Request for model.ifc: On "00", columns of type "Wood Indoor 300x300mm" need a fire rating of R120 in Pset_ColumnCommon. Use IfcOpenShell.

First a look at what the model holds.

```python
import ifcopenshell
import ifcopenshell.util.element

model = ifcopenshell.open("model.ifc")
print(model.schema)
storey = next(s for s in model.by_type("IfcBuildingStorey") if s.Name == "00")
columns = [e for e in ifcopenshell.util.element.get_decomposition(storey) if e.is_a("IfcColumn")]
seen = {}
for e in columns:
    element_type = ifcopenshell.util.element.get_type(e)
    key = (element_type.Name if element_type != e and element_type else None, ifcopenshell.util.element.get_pset(e, "Pset_ColumnCommon", "FireRating"))
    seen[key] = seen.get(key, 0) + 1
for (name, value), count in sorted(seen.items(), key=str):
    print(count, "x", name, "|", value)
```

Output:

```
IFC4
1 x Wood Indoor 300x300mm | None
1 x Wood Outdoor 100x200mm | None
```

```python
import ifcopenshell
import ifcopenshell.api.pset
import ifcopenshell.util.element

model = ifcopenshell.open("model.ifc")

storey = next(s for s in model.by_type("IfcBuildingStorey") if s.Name == "00")
columns = [e for e in ifcopenshell.util.element.get_decomposition(storey) if e.is_a("IfcColumn")]

count = 0
for e in columns:
    element_type = ifcopenshell.util.element.get_type(e)
    if element_type in (None, e) or element_type.Name != "Wood Indoor 300x300mm":
        continue
    # add_pset returns the element's existing set when there is one.
    pset = ifcopenshell.api.pset.add_pset(model, product=e, name="Pset_ColumnCommon")
    ifcopenshell.api.pset.edit_pset(model, pset=pset, properties={"FireRating": "R120"})
    count += 1

print(count, "columns updated")

model.write("model-out.ifc")
```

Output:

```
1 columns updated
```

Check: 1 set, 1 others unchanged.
